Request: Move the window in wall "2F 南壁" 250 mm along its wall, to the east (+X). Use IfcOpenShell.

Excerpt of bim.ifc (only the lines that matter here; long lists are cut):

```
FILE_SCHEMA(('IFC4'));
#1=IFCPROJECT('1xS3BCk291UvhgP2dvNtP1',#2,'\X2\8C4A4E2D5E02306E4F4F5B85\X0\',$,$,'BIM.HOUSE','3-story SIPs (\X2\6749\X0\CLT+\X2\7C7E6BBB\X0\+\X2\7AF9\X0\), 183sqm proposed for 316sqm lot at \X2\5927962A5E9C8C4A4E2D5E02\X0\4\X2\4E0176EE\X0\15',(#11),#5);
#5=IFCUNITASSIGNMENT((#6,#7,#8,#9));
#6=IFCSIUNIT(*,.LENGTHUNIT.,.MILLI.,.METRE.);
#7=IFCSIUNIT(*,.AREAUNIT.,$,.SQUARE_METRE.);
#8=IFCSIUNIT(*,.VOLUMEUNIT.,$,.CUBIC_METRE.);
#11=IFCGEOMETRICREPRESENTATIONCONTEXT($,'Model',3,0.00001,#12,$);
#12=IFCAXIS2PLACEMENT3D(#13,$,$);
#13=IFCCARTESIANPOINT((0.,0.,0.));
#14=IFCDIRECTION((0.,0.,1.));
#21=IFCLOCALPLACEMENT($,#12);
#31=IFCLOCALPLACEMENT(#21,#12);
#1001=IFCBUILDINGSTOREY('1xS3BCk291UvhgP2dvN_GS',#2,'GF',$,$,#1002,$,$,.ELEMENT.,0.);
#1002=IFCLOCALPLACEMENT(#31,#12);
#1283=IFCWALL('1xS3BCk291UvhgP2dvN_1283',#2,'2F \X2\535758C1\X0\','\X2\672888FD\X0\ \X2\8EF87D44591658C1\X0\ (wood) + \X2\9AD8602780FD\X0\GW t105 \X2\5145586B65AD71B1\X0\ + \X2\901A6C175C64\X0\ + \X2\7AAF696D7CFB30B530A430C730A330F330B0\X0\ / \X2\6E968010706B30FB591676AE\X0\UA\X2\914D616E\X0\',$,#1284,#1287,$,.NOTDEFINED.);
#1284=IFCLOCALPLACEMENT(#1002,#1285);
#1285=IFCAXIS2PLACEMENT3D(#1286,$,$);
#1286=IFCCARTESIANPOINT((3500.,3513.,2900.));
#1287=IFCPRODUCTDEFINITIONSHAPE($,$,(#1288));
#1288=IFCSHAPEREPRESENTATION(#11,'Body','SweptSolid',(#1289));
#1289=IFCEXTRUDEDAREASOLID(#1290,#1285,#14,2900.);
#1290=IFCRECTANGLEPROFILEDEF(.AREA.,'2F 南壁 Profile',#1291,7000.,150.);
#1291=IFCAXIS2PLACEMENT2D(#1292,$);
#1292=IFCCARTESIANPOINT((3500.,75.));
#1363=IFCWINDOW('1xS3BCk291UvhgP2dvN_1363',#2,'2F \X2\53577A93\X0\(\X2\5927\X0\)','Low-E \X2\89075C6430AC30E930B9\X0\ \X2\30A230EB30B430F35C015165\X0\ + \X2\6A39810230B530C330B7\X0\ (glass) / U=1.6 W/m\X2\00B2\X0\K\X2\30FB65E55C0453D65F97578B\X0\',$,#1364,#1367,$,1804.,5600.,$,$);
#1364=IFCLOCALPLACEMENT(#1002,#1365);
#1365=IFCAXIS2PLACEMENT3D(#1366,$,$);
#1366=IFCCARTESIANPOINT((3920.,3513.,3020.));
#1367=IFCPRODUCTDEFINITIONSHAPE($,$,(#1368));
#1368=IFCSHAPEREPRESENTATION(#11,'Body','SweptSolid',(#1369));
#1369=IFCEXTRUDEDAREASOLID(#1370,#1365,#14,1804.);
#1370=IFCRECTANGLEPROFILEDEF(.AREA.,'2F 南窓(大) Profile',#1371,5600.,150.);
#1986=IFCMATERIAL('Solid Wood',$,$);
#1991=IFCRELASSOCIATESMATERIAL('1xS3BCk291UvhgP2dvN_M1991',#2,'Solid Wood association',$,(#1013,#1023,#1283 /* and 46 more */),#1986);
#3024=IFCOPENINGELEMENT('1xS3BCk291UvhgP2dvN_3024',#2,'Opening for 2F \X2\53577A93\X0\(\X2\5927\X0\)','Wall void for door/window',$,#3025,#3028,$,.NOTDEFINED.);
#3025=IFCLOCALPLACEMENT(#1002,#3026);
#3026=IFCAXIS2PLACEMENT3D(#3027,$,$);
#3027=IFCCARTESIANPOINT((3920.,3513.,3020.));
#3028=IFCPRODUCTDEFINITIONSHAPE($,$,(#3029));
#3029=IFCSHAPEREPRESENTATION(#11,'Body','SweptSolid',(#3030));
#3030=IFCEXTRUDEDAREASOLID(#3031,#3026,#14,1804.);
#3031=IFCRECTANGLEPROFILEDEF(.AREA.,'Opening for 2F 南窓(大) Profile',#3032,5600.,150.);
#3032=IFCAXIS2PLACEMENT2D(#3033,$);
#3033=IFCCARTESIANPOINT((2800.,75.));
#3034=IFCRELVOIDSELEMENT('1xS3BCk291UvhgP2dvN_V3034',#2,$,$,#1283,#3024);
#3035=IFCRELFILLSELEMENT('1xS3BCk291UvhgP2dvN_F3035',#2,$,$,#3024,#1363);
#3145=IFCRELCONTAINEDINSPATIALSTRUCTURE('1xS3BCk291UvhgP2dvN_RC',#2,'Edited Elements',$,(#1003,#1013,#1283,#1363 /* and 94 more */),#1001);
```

```python
import ifcopenshell
import ifcopenshell.api.geometry
import ifcopenshell.util.placement
import ifcopenshell.util.unit

model = ifcopenshell.open("bim.ifc")
unit_scale = ifcopenshell.util.unit.calculate_unit_scale(model)

window = model.by_id(1363)
opening = window.FillsVoids[0].RelatingOpeningElement
wall = opening.VoidsElements[0].RelatingBuildingElement

wall_matrix = ifcopenshell.util.placement.get_local_placement(wall.ObjectPlacement)
shift = wall_matrix[:3, 0] * 0.25 / unit_scale
before = ifcopenshell.util.placement.get_local_placement(window.ObjectPlacement)[:3, 3].copy()

# The window is not placed relative to its opening, so move both.
for product in (opening, window):
    matrix = ifcopenshell.util.placement.get_local_placement(product.ObjectPlacement)
    matrix[:3, 3] += shift
    ifcopenshell.api.geometry.edit_object_placement(model, product=product, matrix=matrix, is_si=False)

after = ifcopenshell.util.placement.get_local_placement(window.ObjectPlacement)[:3, 3]
print("window moved by", (after - before).round(3) + 0.0)

model.write("bim_v2.ifc")
```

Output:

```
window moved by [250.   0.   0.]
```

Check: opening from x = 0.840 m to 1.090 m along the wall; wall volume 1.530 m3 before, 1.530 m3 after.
